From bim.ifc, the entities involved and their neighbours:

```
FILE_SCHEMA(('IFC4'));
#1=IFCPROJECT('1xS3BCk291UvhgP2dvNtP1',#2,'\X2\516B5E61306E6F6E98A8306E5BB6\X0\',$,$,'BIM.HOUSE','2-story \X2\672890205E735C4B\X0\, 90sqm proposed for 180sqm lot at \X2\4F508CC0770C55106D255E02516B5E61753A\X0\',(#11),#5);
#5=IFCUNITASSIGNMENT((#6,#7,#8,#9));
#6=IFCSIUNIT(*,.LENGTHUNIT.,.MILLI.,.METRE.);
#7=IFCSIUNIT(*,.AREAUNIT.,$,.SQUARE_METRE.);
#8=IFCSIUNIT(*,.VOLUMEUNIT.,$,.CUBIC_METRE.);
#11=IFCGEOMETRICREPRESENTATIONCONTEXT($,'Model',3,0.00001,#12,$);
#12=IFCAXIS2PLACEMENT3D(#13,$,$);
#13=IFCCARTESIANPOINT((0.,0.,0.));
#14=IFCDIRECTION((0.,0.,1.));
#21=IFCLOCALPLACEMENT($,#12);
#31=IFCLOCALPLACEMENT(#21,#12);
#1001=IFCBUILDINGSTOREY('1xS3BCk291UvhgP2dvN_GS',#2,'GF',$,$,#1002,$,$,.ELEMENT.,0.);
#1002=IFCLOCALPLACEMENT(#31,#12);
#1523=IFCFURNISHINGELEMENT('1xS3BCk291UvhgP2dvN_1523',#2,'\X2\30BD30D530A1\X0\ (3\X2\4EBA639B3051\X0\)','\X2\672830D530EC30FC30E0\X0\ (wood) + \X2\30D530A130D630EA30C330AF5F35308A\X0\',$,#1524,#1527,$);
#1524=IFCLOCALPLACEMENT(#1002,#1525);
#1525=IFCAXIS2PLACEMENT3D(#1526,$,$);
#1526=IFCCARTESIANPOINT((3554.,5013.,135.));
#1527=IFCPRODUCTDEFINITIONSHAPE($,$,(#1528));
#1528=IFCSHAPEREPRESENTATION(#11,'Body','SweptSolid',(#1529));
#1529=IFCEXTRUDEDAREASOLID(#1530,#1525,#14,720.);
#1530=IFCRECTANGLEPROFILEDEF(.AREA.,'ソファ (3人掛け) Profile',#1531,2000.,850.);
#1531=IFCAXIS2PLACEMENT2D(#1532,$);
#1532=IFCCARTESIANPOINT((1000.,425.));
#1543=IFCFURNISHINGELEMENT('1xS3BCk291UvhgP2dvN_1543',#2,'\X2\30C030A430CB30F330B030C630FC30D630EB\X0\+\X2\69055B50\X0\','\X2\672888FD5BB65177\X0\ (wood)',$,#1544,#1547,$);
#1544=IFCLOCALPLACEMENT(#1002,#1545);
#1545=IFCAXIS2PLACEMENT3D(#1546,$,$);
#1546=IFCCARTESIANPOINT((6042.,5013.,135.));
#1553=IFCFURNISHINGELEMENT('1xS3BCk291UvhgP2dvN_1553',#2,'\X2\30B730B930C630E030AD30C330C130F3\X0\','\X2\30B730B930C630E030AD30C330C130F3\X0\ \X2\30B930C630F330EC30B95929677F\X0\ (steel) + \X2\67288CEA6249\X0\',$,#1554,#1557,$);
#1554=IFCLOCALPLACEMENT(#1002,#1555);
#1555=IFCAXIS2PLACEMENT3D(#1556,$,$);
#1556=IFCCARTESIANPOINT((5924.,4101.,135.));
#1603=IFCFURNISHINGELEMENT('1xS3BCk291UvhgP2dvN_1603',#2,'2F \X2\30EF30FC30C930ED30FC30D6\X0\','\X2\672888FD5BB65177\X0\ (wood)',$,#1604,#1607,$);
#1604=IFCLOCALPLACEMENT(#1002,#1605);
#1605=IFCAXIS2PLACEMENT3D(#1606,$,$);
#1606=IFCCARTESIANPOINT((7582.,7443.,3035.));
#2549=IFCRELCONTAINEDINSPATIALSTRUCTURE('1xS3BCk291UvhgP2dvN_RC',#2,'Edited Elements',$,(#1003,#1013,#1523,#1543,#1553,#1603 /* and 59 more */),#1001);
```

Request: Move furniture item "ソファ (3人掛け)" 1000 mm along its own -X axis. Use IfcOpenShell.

```python
import ifcopenshell
import ifcopenshell.api.geometry
import ifcopenshell.util.placement
import ifcopenshell.util.unit

model = ifcopenshell.open("bim.ifc")
unit_scale = ifcopenshell.util.unit.calculate_unit_scale(model)

item = model.by_guid("1xS3BCk291UvhgP2dvN_1523")
matrix = ifcopenshell.util.placement.get_local_placement(item.ObjectPlacement)
matrix[:3, 3] -= matrix[:3, 0] * 1 / unit_scale
ifcopenshell.api.geometry.edit_object_placement(model, product=item, matrix=matrix, is_si=False)

print(ifcopenshell.util.placement.get_local_placement(item.ObjectPlacement).round(3) + 0.0)

model.write("bim_updated.ifc")
```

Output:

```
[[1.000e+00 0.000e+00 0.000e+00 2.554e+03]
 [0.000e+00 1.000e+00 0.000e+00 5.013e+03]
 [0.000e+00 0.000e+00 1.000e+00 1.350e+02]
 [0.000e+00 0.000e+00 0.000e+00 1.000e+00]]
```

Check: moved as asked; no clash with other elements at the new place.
